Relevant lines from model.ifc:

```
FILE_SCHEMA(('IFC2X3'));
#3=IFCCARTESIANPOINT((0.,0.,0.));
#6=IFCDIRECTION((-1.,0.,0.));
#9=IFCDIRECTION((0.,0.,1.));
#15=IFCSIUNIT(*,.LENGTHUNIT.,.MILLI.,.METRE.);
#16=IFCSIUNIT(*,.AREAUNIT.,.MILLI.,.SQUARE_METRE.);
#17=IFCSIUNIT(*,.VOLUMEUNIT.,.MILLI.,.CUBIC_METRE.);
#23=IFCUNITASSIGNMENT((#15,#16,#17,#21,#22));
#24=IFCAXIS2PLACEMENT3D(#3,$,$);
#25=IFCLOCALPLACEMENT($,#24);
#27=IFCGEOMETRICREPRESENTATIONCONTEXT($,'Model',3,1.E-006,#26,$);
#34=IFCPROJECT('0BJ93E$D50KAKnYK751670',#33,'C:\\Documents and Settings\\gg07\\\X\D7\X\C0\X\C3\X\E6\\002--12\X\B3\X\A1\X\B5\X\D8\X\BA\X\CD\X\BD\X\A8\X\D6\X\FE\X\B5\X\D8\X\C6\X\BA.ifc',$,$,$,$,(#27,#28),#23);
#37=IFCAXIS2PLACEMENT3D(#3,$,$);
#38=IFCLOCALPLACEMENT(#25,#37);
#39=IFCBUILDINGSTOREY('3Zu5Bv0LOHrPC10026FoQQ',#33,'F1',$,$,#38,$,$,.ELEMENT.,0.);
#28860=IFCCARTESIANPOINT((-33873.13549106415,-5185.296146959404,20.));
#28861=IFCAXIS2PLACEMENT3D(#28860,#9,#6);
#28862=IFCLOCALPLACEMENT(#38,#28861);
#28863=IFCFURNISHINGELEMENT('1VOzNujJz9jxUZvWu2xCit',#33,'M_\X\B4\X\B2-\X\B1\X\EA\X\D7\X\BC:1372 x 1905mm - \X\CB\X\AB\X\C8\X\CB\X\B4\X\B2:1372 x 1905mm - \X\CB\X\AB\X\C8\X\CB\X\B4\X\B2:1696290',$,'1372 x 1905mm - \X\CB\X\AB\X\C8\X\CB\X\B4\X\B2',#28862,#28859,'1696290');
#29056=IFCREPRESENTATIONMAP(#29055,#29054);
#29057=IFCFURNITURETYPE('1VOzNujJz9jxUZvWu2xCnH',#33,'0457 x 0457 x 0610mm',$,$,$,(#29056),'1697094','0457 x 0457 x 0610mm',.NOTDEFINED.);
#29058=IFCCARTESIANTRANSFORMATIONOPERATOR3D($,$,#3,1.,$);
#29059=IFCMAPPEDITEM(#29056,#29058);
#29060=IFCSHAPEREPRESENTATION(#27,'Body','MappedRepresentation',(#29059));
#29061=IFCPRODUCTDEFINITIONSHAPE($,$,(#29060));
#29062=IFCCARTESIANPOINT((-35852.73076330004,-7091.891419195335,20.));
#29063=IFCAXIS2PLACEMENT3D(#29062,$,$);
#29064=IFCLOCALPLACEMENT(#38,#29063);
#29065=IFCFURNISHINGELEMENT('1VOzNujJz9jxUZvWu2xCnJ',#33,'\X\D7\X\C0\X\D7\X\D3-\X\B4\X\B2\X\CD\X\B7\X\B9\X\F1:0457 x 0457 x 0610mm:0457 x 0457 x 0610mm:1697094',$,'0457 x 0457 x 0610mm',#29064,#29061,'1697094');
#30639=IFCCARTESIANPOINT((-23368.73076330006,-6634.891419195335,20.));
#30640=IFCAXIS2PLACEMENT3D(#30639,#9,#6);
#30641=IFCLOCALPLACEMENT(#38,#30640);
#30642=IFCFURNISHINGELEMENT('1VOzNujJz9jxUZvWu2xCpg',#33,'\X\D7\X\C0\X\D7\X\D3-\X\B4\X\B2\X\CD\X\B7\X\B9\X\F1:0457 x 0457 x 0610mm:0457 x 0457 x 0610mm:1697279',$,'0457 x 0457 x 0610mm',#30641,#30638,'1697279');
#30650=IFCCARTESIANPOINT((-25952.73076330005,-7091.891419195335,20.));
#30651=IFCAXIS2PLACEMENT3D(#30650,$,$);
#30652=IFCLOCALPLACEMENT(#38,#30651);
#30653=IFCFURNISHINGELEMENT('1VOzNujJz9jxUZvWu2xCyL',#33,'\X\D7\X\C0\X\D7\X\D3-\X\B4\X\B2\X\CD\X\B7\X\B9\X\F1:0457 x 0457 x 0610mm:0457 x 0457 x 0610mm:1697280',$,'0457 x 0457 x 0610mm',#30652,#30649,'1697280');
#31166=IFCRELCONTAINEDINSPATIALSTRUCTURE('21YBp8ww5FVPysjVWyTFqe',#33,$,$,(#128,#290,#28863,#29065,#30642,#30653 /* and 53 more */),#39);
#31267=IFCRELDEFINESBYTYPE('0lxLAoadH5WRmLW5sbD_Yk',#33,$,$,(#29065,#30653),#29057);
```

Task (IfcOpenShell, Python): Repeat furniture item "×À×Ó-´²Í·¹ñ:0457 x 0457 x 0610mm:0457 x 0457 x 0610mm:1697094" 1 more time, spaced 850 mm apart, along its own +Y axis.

```python
import ifcopenshell
import ifcopenshell.api.geometry
import ifcopenshell.api.root
import ifcopenshell.util.element
import ifcopenshell.util.placement
import ifcopenshell.util.unit

model = ifcopenshell.open("model.ifc")
unit_scale = ifcopenshell.util.unit.calculate_unit_scale(model)


def reuse_history(source, copy):
    """copy_class also copies each property set's owner history, people and application; keep the originals."""
    for rel in copy.IsDefinedBy:
        if rel.is_a("IfcRelDefinesByProperties") and (history := rel.RelatingPropertyDefinition.OwnerHistory):
            rel.RelatingPropertyDefinition.OwnerHistory = source.OwnerHistory
            ifcopenshell.util.element.remove_deep2(model, history)


source = model.by_guid("1VOzNujJz9jxUZvWu2xCnJ")
base = ifcopenshell.util.placement.get_local_placement(source.ObjectPlacement)
step = base[:3, 1] * 0.85 / unit_scale

for i in range(1, 2):
    copy = ifcopenshell.api.root.copy_class(model, product=source)
    copy.Representation = ifcopenshell.util.element.copy_deep(
        model, source.Representation, exclude=["IfcGeometricRepresentationContext", "IfcRepresentationMap"]
    )
    copy.Name = "×À×Ó-´²Í·¹ñ:0457 x 0457 x 0610mm:0457 x 0457 x 0610mm"
    copy.Tag = None
    reuse_history(source, copy)
    matrix = base.copy()
    matrix[:3, 3] += i * step
    print("added at", matrix[:3, 3].round(3) + 0.0)
    ifcopenshell.api.geometry.edit_object_placement(model, product=copy, matrix=matrix, is_si=False)

model.write("model_rev.ifc")
```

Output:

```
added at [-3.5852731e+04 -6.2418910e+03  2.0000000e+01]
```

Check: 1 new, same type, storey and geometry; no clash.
